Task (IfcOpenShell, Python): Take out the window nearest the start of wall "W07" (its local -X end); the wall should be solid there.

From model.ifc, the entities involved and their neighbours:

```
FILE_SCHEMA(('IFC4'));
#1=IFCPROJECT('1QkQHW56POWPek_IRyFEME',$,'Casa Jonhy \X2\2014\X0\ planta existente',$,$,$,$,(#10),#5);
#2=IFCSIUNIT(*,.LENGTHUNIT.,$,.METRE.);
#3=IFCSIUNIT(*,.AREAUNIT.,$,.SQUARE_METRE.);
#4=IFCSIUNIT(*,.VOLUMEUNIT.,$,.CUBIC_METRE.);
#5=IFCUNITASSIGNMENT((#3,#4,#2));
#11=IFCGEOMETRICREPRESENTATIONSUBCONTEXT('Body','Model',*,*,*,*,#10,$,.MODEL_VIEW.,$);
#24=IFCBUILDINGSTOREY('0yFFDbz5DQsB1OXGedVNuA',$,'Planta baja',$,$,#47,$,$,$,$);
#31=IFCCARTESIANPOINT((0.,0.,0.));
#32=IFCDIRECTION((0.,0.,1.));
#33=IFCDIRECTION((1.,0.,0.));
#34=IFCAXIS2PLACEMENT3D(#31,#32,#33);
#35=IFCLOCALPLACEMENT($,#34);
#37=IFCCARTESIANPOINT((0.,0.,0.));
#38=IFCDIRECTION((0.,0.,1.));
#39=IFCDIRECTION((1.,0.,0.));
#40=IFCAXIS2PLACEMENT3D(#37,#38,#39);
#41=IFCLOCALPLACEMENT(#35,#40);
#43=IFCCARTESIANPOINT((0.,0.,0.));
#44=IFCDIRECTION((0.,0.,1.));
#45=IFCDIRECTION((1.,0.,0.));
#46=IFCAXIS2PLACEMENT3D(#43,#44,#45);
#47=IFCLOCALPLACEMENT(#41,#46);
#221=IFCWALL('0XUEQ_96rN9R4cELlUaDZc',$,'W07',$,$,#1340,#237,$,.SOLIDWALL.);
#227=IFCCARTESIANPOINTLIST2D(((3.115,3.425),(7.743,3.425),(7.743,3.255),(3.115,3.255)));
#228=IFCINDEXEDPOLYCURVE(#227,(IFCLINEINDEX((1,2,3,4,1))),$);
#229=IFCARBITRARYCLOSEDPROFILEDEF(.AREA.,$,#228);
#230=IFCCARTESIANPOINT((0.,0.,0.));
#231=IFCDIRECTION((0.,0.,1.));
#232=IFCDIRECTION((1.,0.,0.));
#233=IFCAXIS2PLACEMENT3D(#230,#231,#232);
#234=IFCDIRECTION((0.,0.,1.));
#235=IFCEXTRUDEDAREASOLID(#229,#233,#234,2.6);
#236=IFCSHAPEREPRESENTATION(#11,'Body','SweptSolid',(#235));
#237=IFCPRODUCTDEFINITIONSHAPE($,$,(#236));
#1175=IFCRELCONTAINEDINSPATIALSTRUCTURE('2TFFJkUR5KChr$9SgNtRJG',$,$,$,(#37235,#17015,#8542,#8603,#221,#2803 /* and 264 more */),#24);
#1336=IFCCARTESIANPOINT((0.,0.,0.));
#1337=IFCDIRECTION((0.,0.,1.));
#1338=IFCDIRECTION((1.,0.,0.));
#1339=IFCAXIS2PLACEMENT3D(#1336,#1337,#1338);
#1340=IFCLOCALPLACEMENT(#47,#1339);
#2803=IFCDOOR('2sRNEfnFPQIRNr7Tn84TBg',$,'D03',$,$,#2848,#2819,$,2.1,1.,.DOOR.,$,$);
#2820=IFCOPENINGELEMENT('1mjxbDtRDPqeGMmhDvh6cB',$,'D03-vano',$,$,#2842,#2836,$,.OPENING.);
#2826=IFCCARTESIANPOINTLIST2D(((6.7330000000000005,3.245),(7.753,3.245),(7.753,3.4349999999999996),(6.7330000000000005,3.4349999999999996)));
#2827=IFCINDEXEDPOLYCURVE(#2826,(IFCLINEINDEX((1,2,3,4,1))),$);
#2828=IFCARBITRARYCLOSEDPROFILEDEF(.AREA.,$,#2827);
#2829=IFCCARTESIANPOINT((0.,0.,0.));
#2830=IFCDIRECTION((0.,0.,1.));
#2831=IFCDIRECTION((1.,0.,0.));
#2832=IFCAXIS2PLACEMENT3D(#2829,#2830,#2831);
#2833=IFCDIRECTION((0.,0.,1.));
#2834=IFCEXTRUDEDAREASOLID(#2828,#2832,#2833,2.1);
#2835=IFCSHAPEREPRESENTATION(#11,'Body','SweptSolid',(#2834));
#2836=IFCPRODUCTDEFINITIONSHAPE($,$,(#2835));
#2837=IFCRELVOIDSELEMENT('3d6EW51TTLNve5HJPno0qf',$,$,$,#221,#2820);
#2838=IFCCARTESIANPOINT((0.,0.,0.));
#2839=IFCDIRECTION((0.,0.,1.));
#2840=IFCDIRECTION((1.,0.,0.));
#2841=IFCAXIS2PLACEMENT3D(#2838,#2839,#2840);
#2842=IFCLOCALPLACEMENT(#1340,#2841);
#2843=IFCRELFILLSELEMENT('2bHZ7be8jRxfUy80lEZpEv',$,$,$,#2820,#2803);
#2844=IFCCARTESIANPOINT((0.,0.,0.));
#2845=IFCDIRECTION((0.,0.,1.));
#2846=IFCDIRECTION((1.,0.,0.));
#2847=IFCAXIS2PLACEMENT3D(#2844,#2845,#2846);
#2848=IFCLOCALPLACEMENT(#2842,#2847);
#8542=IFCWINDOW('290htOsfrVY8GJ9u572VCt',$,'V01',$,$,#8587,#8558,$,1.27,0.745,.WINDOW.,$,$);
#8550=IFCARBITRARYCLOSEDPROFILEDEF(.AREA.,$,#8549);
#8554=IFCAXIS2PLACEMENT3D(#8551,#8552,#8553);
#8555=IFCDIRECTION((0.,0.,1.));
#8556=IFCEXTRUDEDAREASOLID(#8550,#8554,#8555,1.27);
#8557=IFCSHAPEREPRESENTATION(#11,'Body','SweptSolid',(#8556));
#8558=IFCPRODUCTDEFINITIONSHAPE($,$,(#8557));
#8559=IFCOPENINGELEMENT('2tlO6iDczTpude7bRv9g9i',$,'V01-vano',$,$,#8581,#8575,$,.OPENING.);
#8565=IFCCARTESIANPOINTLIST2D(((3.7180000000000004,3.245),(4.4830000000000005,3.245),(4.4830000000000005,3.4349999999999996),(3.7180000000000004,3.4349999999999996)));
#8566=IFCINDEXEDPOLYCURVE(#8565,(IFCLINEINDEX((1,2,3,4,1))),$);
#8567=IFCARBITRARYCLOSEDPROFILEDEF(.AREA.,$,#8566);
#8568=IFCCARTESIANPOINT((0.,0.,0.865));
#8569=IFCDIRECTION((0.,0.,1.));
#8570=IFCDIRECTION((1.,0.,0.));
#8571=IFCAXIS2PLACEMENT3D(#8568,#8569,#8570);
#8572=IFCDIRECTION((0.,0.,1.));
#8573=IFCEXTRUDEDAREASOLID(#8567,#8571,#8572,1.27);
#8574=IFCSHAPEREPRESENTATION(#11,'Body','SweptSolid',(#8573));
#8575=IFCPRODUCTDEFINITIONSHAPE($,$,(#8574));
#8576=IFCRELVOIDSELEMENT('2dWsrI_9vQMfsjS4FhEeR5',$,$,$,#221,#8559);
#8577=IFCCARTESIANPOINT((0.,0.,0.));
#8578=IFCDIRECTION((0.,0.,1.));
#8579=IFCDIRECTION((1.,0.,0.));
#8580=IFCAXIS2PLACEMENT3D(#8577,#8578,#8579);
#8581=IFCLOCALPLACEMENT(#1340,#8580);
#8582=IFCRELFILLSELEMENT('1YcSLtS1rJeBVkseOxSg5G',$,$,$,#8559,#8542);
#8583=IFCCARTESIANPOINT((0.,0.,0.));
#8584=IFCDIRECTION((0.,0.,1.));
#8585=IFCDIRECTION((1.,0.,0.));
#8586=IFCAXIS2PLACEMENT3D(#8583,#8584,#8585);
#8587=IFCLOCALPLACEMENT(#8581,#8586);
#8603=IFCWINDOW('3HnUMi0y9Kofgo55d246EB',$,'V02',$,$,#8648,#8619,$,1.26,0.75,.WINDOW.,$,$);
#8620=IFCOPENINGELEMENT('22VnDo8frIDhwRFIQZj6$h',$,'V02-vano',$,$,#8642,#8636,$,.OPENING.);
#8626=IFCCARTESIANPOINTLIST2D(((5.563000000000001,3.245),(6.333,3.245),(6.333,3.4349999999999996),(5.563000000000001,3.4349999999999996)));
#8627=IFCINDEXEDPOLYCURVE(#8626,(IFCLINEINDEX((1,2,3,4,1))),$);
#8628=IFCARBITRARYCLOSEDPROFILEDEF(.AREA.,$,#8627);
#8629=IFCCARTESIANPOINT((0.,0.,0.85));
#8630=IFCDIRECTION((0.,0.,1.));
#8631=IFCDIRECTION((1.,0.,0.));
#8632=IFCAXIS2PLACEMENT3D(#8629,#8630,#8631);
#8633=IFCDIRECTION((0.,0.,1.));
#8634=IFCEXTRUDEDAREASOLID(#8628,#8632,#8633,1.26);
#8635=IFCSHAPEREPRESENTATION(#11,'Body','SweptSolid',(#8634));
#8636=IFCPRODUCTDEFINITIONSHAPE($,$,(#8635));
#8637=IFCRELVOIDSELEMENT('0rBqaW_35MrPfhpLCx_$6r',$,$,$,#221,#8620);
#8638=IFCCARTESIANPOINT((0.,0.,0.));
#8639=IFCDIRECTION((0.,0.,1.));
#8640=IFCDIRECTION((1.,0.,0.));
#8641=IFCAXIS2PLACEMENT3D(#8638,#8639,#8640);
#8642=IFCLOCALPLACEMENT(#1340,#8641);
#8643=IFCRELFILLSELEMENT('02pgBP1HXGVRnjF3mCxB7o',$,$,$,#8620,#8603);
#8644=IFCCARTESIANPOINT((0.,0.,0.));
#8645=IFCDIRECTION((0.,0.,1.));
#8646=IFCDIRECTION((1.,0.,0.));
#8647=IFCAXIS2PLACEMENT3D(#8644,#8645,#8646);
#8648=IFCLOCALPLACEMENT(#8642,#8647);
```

```python
import ifcopenshell
import ifcopenshell.api.feature
import ifcopenshell.api.root
import ifcopenshell.geom
import ifcopenshell.util.shape

model = ifcopenshell.open("model.ifc")
settings = ifcopenshell.geom.settings()


def volume(element):
    """Net volume in cubic metres, openings subtracted."""
    shape = ifcopenshell.geom.create_shape(settings, element)
    return ifcopenshell.util.shape.get_volume(shape.geometry)


window = model.by_guid("290htOsfrVY8GJ9u572VCt")
opening = window.FillsVoids[0].RelatingOpeningElement
wall = opening.VoidsElements[0].RelatingBuildingElement
before = volume(wall)

ifcopenshell.api.root.remove_product(model, product=window)
ifcopenshell.api.feature.remove_feature(model, feature=opening)

after = volume(wall)

print(f"wall volume {before:.3f} -> {after:.3f} m3")

model.write("model-out.ifc")
```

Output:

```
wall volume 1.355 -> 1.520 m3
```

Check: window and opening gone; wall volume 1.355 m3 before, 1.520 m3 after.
